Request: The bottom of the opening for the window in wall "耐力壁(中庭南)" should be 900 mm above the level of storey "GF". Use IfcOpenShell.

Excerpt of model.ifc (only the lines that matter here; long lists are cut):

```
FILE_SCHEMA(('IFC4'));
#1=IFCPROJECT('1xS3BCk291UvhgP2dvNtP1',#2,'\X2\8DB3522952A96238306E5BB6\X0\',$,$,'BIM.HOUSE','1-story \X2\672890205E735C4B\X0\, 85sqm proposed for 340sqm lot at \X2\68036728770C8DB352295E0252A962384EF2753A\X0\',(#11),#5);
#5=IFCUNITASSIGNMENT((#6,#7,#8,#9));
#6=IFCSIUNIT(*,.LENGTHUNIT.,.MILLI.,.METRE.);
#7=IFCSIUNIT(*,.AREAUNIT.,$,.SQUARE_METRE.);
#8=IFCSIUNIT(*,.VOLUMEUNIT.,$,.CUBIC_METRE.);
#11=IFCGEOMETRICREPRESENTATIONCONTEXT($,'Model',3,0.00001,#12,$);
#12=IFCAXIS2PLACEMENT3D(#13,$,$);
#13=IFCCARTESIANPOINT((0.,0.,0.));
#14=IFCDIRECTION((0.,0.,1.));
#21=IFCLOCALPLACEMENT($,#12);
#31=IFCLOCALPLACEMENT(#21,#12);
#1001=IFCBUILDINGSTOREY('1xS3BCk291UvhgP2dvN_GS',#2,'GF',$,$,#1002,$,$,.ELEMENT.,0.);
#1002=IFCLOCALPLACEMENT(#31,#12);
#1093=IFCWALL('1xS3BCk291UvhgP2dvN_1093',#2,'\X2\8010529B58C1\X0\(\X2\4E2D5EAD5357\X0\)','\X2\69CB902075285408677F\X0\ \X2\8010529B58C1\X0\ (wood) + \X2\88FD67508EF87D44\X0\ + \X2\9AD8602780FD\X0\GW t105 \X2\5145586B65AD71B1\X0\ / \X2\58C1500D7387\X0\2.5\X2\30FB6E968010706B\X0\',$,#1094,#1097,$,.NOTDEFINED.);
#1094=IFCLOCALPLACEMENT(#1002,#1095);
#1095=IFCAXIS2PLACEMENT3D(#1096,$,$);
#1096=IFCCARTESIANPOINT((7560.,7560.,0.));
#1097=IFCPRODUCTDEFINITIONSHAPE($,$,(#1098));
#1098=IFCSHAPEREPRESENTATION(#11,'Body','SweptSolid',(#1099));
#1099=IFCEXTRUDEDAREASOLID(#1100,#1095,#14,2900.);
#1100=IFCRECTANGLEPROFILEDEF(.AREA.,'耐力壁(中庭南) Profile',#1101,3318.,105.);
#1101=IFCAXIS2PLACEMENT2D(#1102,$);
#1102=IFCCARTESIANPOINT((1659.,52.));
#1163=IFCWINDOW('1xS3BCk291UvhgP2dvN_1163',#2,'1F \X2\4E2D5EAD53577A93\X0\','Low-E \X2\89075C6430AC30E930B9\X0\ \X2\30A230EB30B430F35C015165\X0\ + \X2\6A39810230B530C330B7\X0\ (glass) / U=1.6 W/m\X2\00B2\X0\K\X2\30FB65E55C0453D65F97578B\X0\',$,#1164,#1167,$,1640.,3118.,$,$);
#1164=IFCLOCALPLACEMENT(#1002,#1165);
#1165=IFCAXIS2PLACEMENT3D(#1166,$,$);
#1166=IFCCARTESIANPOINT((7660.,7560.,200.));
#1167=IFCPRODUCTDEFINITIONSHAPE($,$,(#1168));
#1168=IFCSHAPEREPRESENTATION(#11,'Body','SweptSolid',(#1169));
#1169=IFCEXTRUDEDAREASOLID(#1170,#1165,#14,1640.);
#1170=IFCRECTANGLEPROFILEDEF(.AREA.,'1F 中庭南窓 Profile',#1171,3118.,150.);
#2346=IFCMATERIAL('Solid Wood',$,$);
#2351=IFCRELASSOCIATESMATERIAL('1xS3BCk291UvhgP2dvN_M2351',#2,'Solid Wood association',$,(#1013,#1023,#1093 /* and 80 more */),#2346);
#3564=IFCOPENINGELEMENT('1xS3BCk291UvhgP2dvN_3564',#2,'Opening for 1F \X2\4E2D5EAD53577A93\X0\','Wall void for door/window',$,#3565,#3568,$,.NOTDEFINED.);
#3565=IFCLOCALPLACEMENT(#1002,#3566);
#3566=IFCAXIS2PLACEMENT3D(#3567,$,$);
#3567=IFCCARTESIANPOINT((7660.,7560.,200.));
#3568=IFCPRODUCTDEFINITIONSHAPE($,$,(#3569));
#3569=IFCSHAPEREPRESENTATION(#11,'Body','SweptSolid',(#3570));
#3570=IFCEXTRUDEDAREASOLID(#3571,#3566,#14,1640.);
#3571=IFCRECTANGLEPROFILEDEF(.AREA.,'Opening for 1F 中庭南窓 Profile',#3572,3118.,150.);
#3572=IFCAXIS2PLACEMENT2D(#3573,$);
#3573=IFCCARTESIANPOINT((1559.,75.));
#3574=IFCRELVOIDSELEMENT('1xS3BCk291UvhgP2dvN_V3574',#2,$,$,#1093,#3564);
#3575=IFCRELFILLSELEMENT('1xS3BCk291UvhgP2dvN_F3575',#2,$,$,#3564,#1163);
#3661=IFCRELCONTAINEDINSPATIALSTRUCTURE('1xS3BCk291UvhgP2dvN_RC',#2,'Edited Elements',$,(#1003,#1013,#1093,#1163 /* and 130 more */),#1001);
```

```python
import numpy as np
import ifcopenshell
import ifcopenshell.api.geometry
import ifcopenshell.geom
import ifcopenshell.util.element
import ifcopenshell.util.placement
import ifcopenshell.util.shape
import ifcopenshell.util.unit

model = ifcopenshell.open("model.ifc")
unit_scale = ifcopenshell.util.unit.calculate_unit_scale(model)

window = model.by_guid("1xS3BCk291UvhgP2dvN_1163")
opening = window.FillsVoids[0].RelatingOpeningElement
storey = ifcopenshell.util.element.get_container(window, ifc_class="IfcBuildingStorey")
level = ifcopenshell.util.placement.get_local_placement(storey.ObjectPlacement)[2, 3]

# The opening's origin need not be at the sill, so measure its lowest point.
shape = ifcopenshell.geom.create_shape(ifcopenshell.geom.settings(), opening)
bottom = ifcopenshell.util.shape.get_shape_bottom_elevation(shape, shape.geometry) / unit_scale
dz = level + 0.9 / unit_scale - bottom

shift = np.array([0.0, 0.0, dz])
# The window is not placed relative to its opening, so move both.
for product in (opening, window):
    matrix = ifcopenshell.util.placement.get_local_placement(product.ObjectPlacement)
    matrix[:3, 3] += shift
    ifcopenshell.api.geometry.edit_object_placement(model, product=product, matrix=matrix, is_si=False)

print(f"moved by {dz * unit_scale:+.3f} m")

model.write("model_rev.ifc")
```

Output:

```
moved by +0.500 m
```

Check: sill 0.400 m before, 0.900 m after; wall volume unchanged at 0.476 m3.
